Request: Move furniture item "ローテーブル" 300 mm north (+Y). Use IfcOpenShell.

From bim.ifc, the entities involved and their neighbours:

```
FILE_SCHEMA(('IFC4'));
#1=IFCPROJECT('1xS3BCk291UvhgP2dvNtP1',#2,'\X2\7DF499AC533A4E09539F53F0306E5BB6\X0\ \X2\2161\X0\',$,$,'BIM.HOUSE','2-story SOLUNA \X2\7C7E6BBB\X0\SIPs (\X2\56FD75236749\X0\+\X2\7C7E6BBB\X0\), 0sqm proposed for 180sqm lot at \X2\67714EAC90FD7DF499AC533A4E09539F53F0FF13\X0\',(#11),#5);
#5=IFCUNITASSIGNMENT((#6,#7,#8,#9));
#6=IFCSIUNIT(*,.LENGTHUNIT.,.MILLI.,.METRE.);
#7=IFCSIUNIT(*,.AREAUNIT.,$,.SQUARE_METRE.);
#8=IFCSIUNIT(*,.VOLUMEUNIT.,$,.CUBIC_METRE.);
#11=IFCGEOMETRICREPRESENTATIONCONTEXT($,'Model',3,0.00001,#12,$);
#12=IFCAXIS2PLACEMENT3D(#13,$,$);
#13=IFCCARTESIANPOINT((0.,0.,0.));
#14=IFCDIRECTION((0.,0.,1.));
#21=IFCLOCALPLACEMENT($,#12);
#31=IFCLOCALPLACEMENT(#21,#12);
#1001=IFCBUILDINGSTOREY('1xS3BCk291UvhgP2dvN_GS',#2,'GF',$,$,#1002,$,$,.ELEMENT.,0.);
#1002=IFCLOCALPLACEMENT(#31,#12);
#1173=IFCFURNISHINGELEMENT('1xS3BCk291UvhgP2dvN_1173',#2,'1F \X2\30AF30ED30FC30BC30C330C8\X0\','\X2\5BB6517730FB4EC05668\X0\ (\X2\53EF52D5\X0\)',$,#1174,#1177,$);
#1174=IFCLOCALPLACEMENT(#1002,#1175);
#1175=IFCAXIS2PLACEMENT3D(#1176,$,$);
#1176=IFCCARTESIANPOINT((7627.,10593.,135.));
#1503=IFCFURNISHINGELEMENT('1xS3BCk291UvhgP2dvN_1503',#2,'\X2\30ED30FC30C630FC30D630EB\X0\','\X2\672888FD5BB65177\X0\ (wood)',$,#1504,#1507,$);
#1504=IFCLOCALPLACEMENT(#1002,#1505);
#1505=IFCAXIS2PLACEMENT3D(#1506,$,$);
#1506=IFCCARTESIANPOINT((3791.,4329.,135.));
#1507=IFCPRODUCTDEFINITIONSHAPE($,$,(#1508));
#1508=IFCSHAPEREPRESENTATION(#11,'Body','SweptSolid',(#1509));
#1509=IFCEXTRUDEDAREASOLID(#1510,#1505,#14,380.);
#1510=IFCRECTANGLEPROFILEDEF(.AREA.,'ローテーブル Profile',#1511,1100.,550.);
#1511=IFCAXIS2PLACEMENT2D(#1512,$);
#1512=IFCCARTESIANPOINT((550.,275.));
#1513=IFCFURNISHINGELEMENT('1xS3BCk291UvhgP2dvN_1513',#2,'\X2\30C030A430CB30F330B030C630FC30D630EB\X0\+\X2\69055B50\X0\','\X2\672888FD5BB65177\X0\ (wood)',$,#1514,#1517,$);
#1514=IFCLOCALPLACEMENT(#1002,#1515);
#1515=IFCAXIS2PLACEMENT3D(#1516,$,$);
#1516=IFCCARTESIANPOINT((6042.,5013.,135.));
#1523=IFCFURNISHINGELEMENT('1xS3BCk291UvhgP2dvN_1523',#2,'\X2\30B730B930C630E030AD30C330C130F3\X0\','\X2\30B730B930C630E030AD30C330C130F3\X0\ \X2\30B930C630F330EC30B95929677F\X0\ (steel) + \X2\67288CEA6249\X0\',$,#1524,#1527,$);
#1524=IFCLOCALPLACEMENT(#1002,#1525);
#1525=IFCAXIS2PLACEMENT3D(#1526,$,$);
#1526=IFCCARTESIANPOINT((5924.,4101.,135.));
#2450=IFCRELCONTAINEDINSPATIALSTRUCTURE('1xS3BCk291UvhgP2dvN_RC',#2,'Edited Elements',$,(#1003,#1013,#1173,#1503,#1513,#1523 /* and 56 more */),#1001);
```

```python
import ifcopenshell
import ifcopenshell.api.geometry
import ifcopenshell.util.placement
import ifcopenshell.util.unit

model = ifcopenshell.open("bim.ifc")
unit_scale = ifcopenshell.util.unit.calculate_unit_scale(model)

item = model.by_guid("1xS3BCk291UvhgP2dvN_1503")
matrix = ifcopenshell.util.placement.get_local_placement(item.ObjectPlacement)
matrix[1, 3] += 0.3 / unit_scale
ifcopenshell.api.geometry.edit_object_placement(model, product=item, matrix=matrix, is_si=False)

print(ifcopenshell.util.placement.get_local_placement(item.ObjectPlacement).round(3) + 0.0)

model.write("bim-out.ifc")
```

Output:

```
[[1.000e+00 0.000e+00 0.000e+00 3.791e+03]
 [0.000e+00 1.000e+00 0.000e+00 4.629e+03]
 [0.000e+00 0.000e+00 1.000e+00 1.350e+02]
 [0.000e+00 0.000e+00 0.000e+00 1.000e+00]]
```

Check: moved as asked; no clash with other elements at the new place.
